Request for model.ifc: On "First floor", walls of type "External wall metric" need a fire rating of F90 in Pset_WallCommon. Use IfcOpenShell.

First a look at what the model holds.

```python
import ifcopenshell
import ifcopenshell.util.element

model = ifcopenshell.open("model.ifc")
print(model.schema)
storey = next(s for s in model.by_type("IfcBuildingStorey") if s.Name == "First floor")
walls = [e for e in ifcopenshell.util.element.get_decomposition(storey) if e.is_a("IfcWall")]
seen = {}
for e in walls:
    element_type = ifcopenshell.util.element.get_type(e)
    key = (element_type.Name if element_type != e and element_type else None, ifcopenshell.util.element.get_pset(e, "Pset_WallCommon", "FireRating"))
    seen[key] = seen.get(key, 0) + 1
for (name, value), count in sorted(seen.items(), key=str):
    print(count, "x", name, "|", value)
```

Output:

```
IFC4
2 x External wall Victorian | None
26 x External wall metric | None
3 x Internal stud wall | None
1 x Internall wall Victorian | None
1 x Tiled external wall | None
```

```python
import ifcopenshell
import ifcopenshell.api.pset
import ifcopenshell.util.element

model = ifcopenshell.open("model.ifc")

storey = next(s for s in model.by_type("IfcBuildingStorey") if s.Name == "First floor")
walls = [e for e in ifcopenshell.util.element.get_decomposition(storey) if e.is_a("IfcWall")]

count = 0
for e in walls:
    element_type = ifcopenshell.util.element.get_type(e)
    if element_type in (None, e) or element_type.Name != "External wall metric":
        continue
    # add_pset returns the element's existing set when there is one.
    pset = ifcopenshell.api.pset.add_pset(model, product=e, name="Pset_WallCommon")
    ifcopenshell.api.pset.edit_pset(model, pset=pset, properties={"FireRating": "F90"})
    count += 1

print(count, "walls updated")

model.write("model_rev.ifc")
```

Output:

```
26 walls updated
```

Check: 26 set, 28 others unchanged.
